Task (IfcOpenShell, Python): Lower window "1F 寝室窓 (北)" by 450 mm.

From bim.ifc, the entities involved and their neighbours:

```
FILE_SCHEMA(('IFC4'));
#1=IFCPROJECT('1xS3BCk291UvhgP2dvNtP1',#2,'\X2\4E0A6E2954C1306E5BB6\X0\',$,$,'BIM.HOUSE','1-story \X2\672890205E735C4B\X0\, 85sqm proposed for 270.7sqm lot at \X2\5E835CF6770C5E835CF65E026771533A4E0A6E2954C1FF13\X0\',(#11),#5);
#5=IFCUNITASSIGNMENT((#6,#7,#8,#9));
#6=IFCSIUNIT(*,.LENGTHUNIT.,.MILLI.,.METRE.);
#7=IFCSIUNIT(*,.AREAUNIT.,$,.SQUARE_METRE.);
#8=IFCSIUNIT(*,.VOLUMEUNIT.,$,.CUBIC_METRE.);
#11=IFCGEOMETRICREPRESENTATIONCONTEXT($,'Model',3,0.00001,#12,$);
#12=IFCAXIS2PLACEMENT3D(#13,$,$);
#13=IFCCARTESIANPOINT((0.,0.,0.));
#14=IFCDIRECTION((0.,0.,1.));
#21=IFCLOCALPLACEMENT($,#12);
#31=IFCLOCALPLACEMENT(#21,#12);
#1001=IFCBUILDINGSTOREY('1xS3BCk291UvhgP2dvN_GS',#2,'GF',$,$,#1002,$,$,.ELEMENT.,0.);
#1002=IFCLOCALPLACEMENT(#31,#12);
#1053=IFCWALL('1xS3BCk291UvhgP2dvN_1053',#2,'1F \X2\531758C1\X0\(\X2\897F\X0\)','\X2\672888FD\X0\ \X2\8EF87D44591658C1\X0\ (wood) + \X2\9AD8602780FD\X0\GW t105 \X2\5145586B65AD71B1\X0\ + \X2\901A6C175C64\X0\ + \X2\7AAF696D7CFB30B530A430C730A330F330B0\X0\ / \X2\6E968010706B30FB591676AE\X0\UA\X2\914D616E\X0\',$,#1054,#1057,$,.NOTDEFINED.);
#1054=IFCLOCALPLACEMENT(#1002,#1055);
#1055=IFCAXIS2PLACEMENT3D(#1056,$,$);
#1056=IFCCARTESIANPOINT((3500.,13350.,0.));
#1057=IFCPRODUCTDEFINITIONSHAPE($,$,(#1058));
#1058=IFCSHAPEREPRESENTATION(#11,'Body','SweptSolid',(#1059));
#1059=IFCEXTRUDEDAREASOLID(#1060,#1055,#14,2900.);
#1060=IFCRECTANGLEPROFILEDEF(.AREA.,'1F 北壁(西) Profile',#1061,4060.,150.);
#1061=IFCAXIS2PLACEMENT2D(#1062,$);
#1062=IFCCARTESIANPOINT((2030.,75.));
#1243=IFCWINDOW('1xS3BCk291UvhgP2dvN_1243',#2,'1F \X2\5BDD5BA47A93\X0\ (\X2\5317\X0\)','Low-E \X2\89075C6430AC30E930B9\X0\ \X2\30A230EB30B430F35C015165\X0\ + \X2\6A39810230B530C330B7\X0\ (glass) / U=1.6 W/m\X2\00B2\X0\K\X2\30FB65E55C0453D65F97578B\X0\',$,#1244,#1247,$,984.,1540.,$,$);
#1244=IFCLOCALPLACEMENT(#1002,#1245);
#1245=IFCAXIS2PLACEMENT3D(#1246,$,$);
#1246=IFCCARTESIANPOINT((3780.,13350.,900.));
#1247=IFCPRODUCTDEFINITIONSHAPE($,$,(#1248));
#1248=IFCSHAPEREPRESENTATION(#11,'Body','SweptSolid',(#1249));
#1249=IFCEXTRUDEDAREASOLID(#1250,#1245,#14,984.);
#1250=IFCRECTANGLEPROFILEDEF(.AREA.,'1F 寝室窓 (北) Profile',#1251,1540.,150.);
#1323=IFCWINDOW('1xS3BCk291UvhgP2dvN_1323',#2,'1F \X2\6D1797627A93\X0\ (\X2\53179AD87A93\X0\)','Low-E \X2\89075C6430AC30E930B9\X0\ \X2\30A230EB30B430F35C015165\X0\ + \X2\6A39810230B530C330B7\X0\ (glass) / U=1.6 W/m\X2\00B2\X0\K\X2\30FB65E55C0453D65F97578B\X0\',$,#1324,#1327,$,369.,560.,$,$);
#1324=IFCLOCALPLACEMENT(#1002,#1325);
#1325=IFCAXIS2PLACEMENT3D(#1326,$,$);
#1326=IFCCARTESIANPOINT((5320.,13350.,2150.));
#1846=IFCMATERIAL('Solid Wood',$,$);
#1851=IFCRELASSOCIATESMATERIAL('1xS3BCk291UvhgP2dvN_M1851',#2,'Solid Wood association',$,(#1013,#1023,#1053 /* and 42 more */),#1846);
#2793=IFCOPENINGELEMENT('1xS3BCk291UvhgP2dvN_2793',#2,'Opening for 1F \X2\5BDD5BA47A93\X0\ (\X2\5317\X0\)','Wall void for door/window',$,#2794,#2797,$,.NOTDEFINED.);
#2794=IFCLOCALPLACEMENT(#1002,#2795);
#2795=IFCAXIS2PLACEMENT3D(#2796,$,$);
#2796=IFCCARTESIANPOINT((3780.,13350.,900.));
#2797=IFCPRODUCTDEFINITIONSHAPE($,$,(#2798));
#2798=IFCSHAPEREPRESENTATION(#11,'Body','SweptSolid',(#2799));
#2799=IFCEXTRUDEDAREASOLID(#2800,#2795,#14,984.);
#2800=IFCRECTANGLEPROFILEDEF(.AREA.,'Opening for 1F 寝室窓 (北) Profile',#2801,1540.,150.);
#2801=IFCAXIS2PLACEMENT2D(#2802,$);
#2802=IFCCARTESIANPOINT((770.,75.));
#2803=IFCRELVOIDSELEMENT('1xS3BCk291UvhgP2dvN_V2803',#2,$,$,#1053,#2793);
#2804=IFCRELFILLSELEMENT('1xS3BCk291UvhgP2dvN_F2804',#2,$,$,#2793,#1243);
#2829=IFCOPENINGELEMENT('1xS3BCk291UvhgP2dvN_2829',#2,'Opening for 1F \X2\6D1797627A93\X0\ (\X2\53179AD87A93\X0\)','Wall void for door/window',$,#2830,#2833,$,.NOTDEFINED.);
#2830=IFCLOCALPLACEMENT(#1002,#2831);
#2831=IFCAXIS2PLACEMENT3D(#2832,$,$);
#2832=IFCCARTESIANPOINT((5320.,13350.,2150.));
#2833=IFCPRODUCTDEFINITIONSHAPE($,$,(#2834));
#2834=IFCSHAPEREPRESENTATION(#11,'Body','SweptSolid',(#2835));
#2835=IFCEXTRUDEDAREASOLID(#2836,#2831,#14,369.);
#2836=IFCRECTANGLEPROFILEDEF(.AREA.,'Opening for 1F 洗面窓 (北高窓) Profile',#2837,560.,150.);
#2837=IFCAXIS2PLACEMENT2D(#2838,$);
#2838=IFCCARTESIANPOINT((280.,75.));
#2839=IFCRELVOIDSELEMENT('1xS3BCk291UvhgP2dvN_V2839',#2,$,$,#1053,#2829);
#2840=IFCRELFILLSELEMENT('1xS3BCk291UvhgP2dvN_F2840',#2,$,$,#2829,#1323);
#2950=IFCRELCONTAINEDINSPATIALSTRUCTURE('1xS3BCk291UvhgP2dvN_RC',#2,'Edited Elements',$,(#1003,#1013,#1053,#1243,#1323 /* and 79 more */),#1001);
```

```python
import numpy as np
import ifcopenshell
import ifcopenshell.api.geometry
import ifcopenshell.util.placement
import ifcopenshell.util.unit

model = ifcopenshell.open("bim.ifc")
unit_scale = ifcopenshell.util.unit.calculate_unit_scale(model)

window = model.by_id(1243)
opening = window.FillsVoids[0].RelatingOpeningElement
dz = -450.0

shift = np.array([0.0, 0.0, dz])
# The window is not placed relative to its opening, so move both.
for product in (opening, window):
    matrix = ifcopenshell.util.placement.get_local_placement(product.ObjectPlacement)
    matrix[:3, 3] += shift
    ifcopenshell.api.geometry.edit_object_placement(model, product=product, matrix=matrix, is_si=False)

print(f"moved by {dz * unit_scale:+.3f} m")

model.write("bim_updated.ifc")
```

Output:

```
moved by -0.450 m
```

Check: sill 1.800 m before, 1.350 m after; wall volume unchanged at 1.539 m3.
